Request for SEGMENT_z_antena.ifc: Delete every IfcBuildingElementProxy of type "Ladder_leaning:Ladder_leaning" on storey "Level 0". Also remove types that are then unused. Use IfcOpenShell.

First a look at what the model holds.

```python
import ifcopenshell
import ifcopenshell.util.element

model = ifcopenshell.open("SEGMENT_z_antena.ifc")
print(model.schema)
storey = next(s for s in model.by_type("IfcBuildingStorey") if s.Name == "Level 0")
proxies = [e for e in ifcopenshell.util.element.get_decomposition(storey) if e.is_a("IfcBuildingElementProxy")]
seen = {}
for e in proxies:
    element_type = ifcopenshell.util.element.get_type(e)
    name = element_type.Name if element_type not in (None, e) else None
    seen[name] = seen.get(name, 0) + 1
for name, count in sorted(seen.items(), key=str):
    print(count, "x", name)
```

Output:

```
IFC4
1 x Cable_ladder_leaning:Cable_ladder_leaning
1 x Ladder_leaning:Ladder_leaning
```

```python
import ifcopenshell
import ifcopenshell.api.root
import ifcopenshell.util.element

model = ifcopenshell.open("SEGMENT_z_antena.ifc")

storey = next(s for s in model.by_type("IfcBuildingStorey") if s.Name == "Level 0")
proxies = [e for e in ifcopenshell.util.element.get_decomposition(storey) if e.is_a("IfcBuildingElementProxy")]
targets = [e for e in proxies if (t := ifcopenshell.util.element.get_type(e)) not in (None, e) and t.Name == "Ladder_leaning:Ladder_leaning"]
types = {ifcopenshell.util.element.get_type(e) for e in targets} - {None, *targets}

for e in targets:
    ifcopenshell.api.root.remove_product(model, product=e)
print(len(targets), "removed")

unused = [t for t in types if not ifcopenshell.util.element.get_types(t)]
for t in unused:
    ifcopenshell.api.root.remove_product(model, product=t)
print(len(unused), "unused types removed")

model.write("SEGMENT_z_antena_v2.ifc")
```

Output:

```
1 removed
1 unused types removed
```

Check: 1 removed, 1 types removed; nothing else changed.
